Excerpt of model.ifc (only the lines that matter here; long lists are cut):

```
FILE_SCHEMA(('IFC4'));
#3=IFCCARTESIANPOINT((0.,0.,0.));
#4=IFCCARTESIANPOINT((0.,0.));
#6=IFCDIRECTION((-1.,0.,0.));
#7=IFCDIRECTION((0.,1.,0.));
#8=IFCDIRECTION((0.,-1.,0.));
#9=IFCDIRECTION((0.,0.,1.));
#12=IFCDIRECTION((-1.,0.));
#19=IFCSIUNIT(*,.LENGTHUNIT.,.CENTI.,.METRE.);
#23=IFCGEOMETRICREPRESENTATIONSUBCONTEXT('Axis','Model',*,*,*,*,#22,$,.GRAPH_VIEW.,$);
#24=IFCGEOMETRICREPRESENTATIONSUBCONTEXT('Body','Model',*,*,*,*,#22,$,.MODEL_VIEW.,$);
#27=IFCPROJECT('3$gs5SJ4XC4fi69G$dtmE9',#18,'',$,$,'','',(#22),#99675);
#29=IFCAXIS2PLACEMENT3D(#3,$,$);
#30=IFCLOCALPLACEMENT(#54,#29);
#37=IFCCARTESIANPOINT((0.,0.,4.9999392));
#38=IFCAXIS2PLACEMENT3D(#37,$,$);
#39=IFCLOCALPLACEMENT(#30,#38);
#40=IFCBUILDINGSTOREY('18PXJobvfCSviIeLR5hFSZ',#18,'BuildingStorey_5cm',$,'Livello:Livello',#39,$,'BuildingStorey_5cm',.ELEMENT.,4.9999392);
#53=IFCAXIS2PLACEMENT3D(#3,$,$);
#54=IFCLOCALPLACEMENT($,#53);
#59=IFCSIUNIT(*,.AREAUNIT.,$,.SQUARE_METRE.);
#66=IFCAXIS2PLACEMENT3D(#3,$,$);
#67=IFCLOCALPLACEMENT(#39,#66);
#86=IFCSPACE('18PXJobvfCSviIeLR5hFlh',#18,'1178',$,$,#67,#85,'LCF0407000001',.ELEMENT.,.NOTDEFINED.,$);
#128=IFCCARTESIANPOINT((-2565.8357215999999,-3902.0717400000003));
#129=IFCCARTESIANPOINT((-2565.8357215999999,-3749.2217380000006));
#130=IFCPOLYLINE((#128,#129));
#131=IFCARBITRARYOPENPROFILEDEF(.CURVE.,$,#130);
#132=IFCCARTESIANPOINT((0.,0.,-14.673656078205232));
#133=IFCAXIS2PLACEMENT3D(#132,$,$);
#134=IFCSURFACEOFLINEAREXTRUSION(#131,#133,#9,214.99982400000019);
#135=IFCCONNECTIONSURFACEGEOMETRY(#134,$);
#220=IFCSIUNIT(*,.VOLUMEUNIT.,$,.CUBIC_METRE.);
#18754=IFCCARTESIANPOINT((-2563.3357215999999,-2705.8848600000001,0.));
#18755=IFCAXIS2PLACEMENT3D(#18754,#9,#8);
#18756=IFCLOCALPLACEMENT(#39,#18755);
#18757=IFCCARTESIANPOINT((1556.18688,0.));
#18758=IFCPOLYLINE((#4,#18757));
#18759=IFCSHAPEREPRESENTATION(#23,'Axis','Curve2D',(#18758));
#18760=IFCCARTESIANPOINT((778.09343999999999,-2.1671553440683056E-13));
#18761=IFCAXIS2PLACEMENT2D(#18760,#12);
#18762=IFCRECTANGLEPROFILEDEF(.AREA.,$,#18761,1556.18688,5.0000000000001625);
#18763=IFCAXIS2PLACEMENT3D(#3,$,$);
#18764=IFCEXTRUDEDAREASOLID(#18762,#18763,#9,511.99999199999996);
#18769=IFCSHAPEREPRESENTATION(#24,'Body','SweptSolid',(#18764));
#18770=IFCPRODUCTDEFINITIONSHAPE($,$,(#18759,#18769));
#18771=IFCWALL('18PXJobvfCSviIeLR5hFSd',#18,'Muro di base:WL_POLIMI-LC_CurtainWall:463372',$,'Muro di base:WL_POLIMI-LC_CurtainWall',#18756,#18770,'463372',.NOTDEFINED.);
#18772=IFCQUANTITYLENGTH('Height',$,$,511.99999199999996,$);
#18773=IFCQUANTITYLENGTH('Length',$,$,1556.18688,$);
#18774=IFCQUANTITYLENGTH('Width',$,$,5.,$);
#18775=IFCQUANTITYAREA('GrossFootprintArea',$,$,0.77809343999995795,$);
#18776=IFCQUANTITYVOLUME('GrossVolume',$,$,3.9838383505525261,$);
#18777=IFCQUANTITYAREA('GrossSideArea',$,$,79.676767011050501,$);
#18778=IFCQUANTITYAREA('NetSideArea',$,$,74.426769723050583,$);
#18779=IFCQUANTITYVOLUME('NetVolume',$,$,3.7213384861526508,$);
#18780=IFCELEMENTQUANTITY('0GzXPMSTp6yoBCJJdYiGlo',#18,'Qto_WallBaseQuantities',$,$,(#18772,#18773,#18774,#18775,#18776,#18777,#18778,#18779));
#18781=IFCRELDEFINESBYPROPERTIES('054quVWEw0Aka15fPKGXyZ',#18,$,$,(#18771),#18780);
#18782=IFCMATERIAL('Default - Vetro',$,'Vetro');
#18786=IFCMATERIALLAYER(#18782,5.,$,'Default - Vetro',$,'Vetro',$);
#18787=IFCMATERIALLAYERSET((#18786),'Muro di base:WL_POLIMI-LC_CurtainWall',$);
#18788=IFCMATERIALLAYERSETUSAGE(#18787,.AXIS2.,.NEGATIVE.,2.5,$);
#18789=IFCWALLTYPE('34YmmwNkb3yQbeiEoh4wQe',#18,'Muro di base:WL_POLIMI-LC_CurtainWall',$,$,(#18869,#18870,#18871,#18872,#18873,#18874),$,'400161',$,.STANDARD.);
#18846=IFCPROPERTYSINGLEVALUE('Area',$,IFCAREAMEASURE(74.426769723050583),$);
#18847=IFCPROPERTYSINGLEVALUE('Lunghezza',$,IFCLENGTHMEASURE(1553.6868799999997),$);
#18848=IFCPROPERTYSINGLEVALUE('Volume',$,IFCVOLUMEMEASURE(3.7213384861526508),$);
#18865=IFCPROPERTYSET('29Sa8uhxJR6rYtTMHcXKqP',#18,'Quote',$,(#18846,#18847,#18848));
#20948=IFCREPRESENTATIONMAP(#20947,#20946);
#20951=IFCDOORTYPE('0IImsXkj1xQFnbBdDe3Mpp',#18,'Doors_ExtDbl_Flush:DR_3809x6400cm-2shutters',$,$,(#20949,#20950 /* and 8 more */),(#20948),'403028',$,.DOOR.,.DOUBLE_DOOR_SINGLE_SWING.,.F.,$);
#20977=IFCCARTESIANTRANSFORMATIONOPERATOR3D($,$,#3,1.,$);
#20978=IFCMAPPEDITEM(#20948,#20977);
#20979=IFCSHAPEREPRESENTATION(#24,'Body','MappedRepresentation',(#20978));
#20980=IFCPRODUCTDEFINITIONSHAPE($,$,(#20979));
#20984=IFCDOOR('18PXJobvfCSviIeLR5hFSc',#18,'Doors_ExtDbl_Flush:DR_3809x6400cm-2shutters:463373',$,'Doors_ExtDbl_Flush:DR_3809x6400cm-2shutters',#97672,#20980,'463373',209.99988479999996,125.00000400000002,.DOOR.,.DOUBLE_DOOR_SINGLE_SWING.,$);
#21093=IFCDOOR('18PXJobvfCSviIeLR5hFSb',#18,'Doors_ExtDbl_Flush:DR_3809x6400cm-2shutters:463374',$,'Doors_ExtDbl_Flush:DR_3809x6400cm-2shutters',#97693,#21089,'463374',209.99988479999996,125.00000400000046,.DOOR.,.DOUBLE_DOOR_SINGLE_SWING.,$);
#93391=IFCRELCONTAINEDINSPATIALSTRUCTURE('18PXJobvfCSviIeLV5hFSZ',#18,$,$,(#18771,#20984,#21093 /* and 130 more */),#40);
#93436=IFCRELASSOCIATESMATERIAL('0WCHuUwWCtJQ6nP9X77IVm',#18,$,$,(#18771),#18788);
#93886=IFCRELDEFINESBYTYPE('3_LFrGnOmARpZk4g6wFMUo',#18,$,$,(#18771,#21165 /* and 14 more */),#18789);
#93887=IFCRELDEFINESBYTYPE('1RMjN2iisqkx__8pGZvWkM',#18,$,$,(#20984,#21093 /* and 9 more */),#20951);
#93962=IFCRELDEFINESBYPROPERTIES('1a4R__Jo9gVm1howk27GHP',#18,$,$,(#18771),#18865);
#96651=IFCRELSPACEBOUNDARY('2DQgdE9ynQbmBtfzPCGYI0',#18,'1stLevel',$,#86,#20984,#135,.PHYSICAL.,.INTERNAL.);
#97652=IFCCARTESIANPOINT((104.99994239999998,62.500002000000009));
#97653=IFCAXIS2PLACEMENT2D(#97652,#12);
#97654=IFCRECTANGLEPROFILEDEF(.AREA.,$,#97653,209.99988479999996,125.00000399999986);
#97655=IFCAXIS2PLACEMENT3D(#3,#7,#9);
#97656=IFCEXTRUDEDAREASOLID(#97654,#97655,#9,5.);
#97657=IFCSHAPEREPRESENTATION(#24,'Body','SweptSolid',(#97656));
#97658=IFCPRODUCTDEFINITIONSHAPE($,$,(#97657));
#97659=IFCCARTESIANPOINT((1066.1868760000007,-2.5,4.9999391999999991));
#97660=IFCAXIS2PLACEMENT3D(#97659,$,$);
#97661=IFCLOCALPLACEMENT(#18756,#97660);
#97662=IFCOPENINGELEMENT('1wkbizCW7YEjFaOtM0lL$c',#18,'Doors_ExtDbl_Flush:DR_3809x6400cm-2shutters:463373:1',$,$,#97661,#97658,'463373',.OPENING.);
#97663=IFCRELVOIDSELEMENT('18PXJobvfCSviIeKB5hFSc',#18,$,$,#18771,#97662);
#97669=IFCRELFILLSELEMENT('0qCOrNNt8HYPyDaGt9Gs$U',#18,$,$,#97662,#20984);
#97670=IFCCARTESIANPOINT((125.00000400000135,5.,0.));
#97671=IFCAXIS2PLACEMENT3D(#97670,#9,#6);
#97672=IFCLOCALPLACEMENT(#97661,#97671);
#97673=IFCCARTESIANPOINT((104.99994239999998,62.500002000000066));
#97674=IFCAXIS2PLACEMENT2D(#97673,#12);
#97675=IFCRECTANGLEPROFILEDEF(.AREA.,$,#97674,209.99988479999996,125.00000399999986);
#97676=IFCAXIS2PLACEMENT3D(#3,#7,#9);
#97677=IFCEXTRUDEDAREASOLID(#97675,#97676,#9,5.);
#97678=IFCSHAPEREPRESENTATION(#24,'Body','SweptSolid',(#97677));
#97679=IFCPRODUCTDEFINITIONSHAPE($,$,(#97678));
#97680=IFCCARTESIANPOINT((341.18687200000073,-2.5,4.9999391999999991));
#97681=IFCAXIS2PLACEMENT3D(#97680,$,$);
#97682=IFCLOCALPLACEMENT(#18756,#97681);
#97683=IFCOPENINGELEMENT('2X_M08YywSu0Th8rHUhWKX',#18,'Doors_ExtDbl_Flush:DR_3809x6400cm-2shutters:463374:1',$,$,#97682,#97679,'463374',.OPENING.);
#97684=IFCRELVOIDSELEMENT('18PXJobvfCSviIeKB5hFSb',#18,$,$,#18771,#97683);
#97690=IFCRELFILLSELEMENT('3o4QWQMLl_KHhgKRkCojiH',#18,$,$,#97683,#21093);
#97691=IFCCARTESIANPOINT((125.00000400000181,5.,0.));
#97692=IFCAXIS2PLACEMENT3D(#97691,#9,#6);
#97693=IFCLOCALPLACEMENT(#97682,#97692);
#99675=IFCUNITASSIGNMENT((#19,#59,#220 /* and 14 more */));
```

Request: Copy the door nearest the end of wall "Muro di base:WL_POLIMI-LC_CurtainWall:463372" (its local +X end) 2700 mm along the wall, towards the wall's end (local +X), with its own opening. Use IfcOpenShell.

```python
import numpy as np
import ifcopenshell
import ifcopenshell.api.feature
import ifcopenshell.api.geometry
import ifcopenshell.api.pset
import ifcopenshell.api.root
import ifcopenshell.geom
import ifcopenshell.util.element
import ifcopenshell.util.placement
import ifcopenshell.util.shape
import ifcopenshell.util.unit

model = ifcopenshell.open("model.ifc")
unit_scale = ifcopenshell.util.unit.calculate_unit_scale(model)
area_scale = ifcopenshell.util.unit.calculate_unit_scale(model, "AREAUNIT")
volume_scale = ifcopenshell.util.unit.calculate_unit_scale(model, "VOLUMEUNIT")
settings = ifcopenshell.geom.settings()


def volume(element):
    """Net volume in cubic metres, openings subtracted."""
    shape = ifcopenshell.geom.create_shape(settings, element)
    return ifcopenshell.util.shape.get_volume(shape.geometry)


def reuse_history(source, copy):
    """copy_class also copies each property set's owner history, people and application; keep the originals."""
    for rel in copy.IsDefinedBy:
        if rel.is_a("IfcRelDefinesByProperties") and (history := rel.RelatingPropertyDefinition.OwnerHistory):
            rel.RelatingPropertyDefinition.OwnerHistory = source.OwnerHistory
            ifcopenshell.util.element.remove_deep2(model, history)


door = model.by_id(20984)
opening = door.FillsVoids[0].RelatingOpeningElement
wall = opening.VoidsElements[0].RelatingBuildingElement
before = volume(wall)
shift = ifcopenshell.util.placement.get_local_placement(wall.ObjectPlacement)[:3, 0] * 2.7 / unit_scale

# copy_class copies the void relationship, type, container and properties, but no geometry.
new_opening = ifcopenshell.api.root.copy_class(model, product=opening)
new_opening.Representation = ifcopenshell.util.element.copy_deep(
    model, opening.Representation, exclude=["IfcGeometricRepresentationContext", "IfcRepresentationMap"]
)
new_opening.Name = "Doors_ExtDbl_Flush:DR_3809x6400cm-2shutters"
new_opening.Tag = None
reuse_history(opening, new_opening)
new_door = ifcopenshell.api.root.copy_class(model, product=door)
new_door.Representation = ifcopenshell.util.element.copy_deep(
    model, door.Representation, exclude=["IfcGeometricRepresentationContext", "IfcRepresentationMap"]
)
new_door.Name = "Doors_ExtDbl_Flush:DR_3809x6400cm-2shutters"
new_door.Tag = None
reuse_history(door, new_door)
ifcopenshell.api.feature.add_filling(model, opening=new_opening, element=new_door)

for old, new in ((opening, new_opening), (door, new_door)):
    matrix = ifcopenshell.util.placement.get_local_placement(old.ObjectPlacement)
    matrix[:3, 3] += shift
    ifcopenshell.api.geometry.edit_object_placement(model, product=new, matrix=matrix, is_si=False)

# The copied space boundaries still share their surfaces with the original.
for rel in new_door.ProvidesBoundaries:
    if rel.ConnectionGeometry:
        rel.ConnectionGeometry = ifcopenshell.util.element.copy_deep(model, rel.ConnectionGeometry)

# Space boundary surfaces are stored in each space's coordinates; move them too.
for rel in new_door.ProvidesBoundaries:
    if not rel.ConnectionGeometry:
        continue
    surface = rel.ConnectionGeometry.SurfaceOnRelatingElement
    space_matrix = ifcopenshell.util.placement.get_local_placement(rel.RelatingSpace.ObjectPlacement)
    point = np.array(surface.Position.Location.Coordinates) + space_matrix[:3, :3].T @ shift
    surface.Position = model.createIfcAxis2Placement3D(
        model.createIfcCartesianPoint(point.tolist()), surface.Position.Axis, surface.Position.RefDirection
    )

after = volume(wall)
thickness = 0.05  # wall thickness in metres

# Update the wall's stored quantities.
qto = model.by_id(ifcopenshell.util.element.get_pset(wall, "Qto_WallBaseQuantities", should_inherit=False)["id"])
ifcopenshell.api.pset.edit_qto(model, qto=qto, properties={
    "NetSideArea": after / thickness / area_scale,
    "NetVolume": after / volume_scale,
})
pset = model.by_id(ifcopenshell.util.element.get_pset(wall, "Quote", should_inherit=False)["id"])
ifcopenshell.api.pset.edit_pset(model, pset=pset, properties={
    "Area": model.create_entity("IfcAreaMeasure", after / thickness / area_scale),
    "Volume": model.create_entity("IfcVolumeMeasure", after / volume_scale),
})

print(f"wall volume {before:.3f} -> {after:.3f} m3")

model.write("model_rev.ifc")
```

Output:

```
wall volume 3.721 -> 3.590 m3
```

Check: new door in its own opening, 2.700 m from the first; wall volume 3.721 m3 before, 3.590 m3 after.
